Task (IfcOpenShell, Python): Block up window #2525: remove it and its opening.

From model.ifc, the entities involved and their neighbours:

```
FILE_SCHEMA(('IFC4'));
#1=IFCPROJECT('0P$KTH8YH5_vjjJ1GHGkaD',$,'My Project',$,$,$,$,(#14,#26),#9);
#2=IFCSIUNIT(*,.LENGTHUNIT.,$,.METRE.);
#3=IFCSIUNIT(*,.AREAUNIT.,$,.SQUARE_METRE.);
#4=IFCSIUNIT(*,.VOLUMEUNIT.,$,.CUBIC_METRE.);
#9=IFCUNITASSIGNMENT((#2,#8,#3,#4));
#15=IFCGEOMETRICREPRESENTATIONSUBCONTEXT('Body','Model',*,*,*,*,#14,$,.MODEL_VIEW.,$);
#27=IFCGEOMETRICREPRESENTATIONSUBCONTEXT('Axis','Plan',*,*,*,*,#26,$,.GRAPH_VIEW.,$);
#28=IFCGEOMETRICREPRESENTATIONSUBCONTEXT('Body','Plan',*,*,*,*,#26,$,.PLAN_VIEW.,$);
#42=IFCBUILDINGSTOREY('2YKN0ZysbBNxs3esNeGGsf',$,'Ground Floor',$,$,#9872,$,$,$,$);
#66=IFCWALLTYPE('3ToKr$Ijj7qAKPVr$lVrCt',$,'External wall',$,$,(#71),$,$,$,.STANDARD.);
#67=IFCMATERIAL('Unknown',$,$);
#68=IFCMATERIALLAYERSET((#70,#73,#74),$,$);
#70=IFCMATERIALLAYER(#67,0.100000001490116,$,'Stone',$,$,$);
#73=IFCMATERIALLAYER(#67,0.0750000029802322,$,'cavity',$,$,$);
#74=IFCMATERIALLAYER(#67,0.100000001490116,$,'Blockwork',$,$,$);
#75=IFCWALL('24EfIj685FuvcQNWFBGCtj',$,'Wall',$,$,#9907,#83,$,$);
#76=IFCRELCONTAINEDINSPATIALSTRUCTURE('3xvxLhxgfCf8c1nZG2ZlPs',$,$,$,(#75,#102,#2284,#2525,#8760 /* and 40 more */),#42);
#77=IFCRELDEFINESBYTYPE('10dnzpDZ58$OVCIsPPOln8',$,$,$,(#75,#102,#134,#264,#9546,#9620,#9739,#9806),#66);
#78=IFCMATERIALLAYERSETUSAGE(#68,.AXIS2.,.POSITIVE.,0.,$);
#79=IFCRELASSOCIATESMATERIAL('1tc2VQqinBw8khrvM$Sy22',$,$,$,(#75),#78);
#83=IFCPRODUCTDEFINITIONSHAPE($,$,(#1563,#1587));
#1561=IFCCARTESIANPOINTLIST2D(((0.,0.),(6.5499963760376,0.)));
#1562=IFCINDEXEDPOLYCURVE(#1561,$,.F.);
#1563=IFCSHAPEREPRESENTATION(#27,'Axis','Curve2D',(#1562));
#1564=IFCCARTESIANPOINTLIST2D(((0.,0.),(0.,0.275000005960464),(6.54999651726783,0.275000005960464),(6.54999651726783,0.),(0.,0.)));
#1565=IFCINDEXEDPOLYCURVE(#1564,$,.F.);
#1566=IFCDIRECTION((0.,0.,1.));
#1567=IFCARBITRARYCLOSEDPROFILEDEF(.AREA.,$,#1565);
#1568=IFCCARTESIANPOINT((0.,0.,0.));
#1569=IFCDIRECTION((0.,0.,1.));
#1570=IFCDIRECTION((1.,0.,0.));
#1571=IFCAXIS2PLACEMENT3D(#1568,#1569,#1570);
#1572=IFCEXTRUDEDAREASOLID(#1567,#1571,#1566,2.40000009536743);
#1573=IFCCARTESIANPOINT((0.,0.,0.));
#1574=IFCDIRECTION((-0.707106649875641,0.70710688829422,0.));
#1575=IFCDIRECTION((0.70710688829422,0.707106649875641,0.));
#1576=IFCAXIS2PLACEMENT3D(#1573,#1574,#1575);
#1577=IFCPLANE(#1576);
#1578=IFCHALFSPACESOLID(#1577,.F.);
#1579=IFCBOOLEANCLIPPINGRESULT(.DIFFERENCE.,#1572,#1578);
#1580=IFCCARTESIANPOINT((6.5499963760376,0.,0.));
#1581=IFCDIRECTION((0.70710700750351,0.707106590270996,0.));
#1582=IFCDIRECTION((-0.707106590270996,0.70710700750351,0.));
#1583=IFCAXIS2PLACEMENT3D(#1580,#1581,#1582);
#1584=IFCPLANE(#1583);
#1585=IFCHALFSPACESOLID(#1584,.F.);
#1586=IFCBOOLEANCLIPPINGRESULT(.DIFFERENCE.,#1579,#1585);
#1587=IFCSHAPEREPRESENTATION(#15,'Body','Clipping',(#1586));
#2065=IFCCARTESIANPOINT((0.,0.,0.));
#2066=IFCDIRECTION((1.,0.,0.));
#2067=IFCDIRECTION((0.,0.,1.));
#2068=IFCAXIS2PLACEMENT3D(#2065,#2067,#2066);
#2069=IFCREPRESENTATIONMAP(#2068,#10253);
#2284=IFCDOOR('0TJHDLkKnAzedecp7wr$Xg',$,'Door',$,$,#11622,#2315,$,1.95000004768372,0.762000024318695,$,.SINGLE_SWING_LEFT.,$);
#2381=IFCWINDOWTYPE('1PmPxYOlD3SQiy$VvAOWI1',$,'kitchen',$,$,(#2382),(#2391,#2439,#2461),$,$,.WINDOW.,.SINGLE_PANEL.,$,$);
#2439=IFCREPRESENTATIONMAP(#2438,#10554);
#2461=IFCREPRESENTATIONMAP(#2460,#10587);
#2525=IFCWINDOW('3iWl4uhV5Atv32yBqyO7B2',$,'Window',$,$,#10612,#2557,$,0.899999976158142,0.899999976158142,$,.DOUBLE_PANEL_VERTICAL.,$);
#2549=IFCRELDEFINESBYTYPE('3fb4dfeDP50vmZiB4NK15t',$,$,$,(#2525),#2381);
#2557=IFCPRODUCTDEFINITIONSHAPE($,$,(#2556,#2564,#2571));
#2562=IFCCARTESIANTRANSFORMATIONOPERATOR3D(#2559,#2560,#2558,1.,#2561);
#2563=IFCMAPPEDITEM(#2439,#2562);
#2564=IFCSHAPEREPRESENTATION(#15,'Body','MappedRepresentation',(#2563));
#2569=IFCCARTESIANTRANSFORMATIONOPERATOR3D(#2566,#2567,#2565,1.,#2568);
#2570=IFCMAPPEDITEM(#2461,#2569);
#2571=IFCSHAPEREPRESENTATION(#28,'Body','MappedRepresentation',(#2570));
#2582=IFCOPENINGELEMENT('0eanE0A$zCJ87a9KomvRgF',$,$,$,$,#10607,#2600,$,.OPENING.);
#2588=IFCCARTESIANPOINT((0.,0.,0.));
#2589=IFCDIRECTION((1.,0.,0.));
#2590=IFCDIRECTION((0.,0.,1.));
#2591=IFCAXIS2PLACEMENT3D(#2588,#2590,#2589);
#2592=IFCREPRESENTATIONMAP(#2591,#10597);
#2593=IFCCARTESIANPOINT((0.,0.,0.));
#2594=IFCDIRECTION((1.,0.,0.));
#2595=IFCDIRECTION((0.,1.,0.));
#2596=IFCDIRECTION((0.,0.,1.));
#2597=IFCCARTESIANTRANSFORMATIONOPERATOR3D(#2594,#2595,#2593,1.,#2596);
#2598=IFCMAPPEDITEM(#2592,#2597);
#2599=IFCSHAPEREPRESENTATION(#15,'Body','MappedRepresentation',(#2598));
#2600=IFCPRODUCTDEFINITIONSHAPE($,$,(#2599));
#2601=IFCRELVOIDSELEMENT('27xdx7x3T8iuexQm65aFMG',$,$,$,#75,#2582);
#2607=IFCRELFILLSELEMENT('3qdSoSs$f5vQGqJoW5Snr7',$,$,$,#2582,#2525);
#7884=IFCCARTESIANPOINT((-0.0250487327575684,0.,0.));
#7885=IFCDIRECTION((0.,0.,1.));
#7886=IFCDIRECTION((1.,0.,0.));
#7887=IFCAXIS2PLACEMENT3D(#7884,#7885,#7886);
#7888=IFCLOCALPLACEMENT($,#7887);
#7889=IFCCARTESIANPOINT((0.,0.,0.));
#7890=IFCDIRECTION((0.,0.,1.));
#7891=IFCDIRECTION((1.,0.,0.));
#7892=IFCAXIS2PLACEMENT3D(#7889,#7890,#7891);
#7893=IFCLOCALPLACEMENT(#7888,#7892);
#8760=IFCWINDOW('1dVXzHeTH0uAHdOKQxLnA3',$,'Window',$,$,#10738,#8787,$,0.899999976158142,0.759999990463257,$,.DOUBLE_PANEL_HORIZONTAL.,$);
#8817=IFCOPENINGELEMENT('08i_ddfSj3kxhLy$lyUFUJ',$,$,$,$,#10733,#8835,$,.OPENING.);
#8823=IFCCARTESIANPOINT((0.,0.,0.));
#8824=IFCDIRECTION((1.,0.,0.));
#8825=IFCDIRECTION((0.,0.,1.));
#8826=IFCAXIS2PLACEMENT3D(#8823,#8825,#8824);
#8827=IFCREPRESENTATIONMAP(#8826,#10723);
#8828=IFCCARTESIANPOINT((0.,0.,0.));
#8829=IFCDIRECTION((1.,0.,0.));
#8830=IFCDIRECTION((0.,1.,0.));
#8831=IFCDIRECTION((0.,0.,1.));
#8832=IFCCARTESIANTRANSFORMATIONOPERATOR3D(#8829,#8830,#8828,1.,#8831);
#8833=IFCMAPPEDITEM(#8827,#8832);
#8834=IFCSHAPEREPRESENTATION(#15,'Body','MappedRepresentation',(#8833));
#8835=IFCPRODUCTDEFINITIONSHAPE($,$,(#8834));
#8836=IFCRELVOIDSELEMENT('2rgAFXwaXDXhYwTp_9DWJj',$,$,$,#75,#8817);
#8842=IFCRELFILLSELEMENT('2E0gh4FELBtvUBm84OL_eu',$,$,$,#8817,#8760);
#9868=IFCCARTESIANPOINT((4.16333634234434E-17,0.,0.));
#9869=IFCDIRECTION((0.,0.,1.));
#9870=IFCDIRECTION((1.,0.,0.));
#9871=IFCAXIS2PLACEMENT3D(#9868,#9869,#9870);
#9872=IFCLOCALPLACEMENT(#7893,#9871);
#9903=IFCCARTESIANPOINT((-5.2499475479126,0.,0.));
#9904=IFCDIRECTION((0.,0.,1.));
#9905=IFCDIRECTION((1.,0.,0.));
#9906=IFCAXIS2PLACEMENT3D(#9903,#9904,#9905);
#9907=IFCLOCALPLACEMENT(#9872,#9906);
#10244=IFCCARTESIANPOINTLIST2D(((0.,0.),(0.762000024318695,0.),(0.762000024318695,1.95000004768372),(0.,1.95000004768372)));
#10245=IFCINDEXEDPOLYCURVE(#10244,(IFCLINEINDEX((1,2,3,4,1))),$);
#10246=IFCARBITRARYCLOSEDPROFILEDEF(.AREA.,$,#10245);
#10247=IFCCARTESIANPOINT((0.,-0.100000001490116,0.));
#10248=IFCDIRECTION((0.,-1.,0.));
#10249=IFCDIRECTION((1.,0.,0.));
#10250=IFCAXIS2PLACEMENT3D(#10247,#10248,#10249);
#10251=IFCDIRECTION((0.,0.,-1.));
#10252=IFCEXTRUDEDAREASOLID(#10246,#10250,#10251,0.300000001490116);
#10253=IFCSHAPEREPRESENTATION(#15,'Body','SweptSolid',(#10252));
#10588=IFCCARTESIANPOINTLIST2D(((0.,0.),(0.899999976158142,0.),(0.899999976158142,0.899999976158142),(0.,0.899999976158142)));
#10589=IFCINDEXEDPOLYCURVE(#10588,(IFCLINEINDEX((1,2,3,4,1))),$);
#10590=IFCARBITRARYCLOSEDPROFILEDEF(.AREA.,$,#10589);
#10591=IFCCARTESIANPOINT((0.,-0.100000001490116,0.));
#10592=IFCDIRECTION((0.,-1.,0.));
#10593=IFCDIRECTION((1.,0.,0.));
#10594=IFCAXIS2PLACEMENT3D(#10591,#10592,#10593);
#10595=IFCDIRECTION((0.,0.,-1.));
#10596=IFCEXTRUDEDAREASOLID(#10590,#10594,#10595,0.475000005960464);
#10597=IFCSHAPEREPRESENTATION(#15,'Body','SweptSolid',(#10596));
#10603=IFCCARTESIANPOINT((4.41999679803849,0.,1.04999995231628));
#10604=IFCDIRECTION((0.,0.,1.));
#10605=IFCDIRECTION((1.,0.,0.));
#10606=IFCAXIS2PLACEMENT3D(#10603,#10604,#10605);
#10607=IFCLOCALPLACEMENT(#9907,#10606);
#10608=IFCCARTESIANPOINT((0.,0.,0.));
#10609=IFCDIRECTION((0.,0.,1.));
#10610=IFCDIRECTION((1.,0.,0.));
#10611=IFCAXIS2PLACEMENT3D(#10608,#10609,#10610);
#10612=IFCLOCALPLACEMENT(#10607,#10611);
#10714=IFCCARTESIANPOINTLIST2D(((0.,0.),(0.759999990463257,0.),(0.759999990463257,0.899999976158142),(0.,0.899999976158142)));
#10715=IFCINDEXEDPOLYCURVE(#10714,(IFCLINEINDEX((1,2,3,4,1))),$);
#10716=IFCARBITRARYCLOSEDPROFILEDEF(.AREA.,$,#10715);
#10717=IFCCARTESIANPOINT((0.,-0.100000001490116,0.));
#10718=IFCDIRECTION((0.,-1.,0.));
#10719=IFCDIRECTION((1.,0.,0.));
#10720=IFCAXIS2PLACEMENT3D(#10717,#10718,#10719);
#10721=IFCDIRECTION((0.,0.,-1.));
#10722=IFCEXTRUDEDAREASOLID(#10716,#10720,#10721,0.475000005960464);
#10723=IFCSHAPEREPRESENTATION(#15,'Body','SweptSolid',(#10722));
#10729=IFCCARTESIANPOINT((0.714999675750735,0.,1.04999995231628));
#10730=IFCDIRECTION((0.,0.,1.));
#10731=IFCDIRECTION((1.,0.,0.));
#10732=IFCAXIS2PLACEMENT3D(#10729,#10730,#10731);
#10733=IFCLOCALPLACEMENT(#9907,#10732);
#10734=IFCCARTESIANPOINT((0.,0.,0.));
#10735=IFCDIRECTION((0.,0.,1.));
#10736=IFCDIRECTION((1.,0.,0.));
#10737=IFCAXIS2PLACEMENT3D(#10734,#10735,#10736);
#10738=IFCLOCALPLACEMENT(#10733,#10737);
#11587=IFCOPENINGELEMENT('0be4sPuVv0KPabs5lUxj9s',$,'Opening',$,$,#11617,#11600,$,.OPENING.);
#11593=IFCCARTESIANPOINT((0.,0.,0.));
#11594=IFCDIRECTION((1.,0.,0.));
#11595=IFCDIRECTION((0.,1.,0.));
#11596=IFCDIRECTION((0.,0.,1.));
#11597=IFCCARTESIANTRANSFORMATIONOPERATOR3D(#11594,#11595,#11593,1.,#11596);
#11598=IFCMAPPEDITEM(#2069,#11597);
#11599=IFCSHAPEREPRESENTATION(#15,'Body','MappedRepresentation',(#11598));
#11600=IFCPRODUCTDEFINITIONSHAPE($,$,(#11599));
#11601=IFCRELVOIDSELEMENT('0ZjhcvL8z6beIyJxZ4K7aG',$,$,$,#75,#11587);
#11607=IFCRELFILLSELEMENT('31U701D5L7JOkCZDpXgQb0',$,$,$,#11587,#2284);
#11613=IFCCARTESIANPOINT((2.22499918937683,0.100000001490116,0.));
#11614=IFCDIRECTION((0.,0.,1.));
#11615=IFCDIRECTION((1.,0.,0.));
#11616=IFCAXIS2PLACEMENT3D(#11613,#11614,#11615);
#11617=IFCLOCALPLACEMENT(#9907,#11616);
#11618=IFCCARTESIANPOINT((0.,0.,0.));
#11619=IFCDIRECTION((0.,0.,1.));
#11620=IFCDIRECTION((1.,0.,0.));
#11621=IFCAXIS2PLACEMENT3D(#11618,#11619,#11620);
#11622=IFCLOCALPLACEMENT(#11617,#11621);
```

```python
import ifcopenshell
import ifcopenshell.api.feature
import ifcopenshell.api.root
import ifcopenshell.geom
import ifcopenshell.util.shape

model = ifcopenshell.open("model.ifc")
settings = ifcopenshell.geom.settings()


def volume(element):
    """Net volume in cubic metres, openings subtracted."""
    shape = ifcopenshell.geom.create_shape(settings, element)
    return ifcopenshell.util.shape.get_volume(shape.geometry)


window = model.by_id(2525)
opening = window.FillsVoids[0].RelatingOpeningElement
wall = opening.VoidsElements[0].RelatingBuildingElement
before = volume(wall)

ifcopenshell.api.root.remove_product(model, product=window)
ifcopenshell.api.feature.remove_feature(model, feature=opening)

after = volume(wall)

print(f"wall volume {before:.3f} -> {after:.3f} m3")

model.write("model_v2.ifc")
```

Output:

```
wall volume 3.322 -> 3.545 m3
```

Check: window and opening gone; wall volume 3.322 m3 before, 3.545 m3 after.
